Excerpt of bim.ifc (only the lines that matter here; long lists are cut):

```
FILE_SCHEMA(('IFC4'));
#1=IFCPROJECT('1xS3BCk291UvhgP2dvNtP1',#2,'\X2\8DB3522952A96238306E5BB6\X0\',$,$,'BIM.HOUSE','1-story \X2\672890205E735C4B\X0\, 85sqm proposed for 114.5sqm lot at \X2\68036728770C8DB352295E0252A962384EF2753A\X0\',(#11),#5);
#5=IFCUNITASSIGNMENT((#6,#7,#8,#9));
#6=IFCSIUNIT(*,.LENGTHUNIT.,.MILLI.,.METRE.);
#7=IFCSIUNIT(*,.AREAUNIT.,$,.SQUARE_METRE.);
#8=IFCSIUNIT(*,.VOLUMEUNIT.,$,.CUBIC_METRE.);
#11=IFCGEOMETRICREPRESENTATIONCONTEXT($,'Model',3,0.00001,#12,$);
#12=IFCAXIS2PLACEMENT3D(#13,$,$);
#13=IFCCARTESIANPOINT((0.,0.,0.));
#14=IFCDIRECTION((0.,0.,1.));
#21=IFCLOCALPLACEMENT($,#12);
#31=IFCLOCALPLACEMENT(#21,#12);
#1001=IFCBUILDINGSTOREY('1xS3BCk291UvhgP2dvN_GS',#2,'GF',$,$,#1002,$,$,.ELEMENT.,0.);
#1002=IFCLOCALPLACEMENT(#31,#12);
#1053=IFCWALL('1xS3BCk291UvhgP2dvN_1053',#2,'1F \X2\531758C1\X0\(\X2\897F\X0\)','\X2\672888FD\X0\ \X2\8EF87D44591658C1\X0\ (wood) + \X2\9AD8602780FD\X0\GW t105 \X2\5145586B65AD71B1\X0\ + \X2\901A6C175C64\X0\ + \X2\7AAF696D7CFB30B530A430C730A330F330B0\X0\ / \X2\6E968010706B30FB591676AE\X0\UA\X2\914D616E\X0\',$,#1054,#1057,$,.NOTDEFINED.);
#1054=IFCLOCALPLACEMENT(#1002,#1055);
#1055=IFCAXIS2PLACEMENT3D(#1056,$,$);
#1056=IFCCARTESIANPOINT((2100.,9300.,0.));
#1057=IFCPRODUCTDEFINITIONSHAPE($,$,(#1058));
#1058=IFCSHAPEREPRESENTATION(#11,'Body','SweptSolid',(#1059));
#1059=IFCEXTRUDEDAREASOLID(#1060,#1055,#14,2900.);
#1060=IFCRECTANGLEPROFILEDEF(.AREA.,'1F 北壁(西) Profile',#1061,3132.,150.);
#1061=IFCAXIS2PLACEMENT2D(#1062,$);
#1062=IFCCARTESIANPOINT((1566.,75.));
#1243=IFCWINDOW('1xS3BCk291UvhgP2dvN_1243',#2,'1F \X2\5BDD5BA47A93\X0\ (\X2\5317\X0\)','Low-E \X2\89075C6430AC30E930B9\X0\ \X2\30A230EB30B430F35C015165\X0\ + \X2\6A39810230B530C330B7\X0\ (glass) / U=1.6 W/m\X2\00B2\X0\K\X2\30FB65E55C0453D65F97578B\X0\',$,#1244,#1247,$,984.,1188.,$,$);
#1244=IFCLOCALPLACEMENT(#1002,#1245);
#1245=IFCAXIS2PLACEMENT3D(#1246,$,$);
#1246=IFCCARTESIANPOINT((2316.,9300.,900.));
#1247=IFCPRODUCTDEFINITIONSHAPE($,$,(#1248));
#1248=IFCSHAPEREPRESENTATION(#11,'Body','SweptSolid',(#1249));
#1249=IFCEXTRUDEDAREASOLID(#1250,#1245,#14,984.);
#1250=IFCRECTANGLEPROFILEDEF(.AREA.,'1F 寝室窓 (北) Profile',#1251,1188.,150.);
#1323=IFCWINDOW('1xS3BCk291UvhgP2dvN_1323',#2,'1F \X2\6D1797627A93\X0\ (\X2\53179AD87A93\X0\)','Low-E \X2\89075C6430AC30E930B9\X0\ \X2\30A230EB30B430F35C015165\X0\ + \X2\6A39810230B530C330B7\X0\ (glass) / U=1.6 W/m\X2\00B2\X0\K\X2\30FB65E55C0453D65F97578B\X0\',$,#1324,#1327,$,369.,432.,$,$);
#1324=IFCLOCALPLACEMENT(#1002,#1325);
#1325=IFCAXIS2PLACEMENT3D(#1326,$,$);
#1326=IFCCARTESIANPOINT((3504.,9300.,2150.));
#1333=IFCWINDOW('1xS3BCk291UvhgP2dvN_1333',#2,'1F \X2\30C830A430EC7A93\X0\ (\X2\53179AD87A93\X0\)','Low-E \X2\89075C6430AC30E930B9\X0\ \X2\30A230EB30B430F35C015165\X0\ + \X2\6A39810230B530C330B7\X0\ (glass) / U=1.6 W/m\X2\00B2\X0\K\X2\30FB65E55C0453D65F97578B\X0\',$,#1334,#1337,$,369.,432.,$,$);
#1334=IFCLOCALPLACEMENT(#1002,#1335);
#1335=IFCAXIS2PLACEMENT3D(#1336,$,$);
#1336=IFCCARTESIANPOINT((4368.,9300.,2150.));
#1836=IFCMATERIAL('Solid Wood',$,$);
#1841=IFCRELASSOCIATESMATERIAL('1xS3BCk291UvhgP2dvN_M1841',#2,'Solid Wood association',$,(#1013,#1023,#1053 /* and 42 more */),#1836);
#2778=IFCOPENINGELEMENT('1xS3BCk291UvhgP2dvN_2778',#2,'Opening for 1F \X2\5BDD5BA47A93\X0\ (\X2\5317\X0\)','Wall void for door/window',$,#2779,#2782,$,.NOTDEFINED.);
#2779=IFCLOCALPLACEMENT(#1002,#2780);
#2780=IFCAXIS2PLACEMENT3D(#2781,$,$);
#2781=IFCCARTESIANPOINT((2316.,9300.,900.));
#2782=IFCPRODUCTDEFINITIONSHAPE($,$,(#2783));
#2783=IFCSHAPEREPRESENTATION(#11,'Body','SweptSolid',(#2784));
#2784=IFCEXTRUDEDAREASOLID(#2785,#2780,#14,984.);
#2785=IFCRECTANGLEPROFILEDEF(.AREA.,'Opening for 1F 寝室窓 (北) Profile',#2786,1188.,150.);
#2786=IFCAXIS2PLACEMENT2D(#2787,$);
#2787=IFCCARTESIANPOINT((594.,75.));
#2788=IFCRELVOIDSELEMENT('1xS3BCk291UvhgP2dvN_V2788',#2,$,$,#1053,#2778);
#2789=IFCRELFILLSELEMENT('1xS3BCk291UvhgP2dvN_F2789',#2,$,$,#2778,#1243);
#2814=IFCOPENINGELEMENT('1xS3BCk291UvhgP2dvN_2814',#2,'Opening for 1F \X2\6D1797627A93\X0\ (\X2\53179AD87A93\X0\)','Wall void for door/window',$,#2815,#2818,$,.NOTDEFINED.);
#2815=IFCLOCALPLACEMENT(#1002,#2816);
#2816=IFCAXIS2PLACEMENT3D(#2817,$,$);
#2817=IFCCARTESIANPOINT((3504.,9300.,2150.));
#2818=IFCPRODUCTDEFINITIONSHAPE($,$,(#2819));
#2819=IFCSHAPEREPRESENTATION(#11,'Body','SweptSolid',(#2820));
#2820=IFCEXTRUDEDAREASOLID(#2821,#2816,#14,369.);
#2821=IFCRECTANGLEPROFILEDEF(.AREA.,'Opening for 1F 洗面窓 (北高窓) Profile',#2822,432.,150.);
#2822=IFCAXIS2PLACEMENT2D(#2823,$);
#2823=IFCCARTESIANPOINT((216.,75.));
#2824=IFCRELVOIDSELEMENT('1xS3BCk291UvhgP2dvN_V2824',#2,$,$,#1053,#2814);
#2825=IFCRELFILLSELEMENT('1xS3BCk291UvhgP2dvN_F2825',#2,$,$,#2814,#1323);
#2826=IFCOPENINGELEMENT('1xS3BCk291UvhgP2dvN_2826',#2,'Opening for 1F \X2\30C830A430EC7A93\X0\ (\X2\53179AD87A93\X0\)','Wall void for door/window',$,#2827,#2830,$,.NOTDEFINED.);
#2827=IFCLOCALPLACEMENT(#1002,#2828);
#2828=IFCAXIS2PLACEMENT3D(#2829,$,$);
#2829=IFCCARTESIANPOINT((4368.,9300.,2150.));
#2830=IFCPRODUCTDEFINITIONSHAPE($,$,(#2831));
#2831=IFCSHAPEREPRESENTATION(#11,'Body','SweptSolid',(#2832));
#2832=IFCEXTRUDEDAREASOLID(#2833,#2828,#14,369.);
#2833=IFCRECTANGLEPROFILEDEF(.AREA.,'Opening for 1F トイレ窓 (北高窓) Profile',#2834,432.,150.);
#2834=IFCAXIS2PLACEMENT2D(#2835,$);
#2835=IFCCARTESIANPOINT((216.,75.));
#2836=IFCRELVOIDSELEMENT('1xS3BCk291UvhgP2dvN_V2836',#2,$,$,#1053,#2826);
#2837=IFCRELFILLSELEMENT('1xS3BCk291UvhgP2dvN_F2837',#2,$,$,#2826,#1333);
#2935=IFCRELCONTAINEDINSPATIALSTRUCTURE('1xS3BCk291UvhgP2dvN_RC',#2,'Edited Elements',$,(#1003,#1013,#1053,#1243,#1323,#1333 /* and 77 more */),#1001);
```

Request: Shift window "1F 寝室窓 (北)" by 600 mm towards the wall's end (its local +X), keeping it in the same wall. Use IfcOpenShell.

```python
import ifcopenshell
import ifcopenshell.api.geometry
import ifcopenshell.util.placement

model = ifcopenshell.open("bim.ifc")

window = model.by_guid("1xS3BCk291UvhgP2dvN_1243")
opening = window.FillsVoids[0].RelatingOpeningElement
wall = opening.VoidsElements[0].RelatingBuildingElement

wall_matrix = ifcopenshell.util.placement.get_local_placement(wall.ObjectPlacement)
shift = wall_matrix[:3, 0] * 600.0
before = ifcopenshell.util.placement.get_local_placement(window.ObjectPlacement)[:3, 3].copy()

# The window is not placed relative to its opening, so move both.
for product in (opening, window):
    matrix = ifcopenshell.util.placement.get_local_placement(product.ObjectPlacement)
    matrix[:3, 3] += shift
    ifcopenshell.api.geometry.edit_object_placement(model, product=product, matrix=matrix, is_si=False)

after = ifcopenshell.util.placement.get_local_placement(window.ObjectPlacement)[:3, 3]
print("window moved by", (after - before).round(3) + 0.0)

model.write("bim_v2.ifc")
```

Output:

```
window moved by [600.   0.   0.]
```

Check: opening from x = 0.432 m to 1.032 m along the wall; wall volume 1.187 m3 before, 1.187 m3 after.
